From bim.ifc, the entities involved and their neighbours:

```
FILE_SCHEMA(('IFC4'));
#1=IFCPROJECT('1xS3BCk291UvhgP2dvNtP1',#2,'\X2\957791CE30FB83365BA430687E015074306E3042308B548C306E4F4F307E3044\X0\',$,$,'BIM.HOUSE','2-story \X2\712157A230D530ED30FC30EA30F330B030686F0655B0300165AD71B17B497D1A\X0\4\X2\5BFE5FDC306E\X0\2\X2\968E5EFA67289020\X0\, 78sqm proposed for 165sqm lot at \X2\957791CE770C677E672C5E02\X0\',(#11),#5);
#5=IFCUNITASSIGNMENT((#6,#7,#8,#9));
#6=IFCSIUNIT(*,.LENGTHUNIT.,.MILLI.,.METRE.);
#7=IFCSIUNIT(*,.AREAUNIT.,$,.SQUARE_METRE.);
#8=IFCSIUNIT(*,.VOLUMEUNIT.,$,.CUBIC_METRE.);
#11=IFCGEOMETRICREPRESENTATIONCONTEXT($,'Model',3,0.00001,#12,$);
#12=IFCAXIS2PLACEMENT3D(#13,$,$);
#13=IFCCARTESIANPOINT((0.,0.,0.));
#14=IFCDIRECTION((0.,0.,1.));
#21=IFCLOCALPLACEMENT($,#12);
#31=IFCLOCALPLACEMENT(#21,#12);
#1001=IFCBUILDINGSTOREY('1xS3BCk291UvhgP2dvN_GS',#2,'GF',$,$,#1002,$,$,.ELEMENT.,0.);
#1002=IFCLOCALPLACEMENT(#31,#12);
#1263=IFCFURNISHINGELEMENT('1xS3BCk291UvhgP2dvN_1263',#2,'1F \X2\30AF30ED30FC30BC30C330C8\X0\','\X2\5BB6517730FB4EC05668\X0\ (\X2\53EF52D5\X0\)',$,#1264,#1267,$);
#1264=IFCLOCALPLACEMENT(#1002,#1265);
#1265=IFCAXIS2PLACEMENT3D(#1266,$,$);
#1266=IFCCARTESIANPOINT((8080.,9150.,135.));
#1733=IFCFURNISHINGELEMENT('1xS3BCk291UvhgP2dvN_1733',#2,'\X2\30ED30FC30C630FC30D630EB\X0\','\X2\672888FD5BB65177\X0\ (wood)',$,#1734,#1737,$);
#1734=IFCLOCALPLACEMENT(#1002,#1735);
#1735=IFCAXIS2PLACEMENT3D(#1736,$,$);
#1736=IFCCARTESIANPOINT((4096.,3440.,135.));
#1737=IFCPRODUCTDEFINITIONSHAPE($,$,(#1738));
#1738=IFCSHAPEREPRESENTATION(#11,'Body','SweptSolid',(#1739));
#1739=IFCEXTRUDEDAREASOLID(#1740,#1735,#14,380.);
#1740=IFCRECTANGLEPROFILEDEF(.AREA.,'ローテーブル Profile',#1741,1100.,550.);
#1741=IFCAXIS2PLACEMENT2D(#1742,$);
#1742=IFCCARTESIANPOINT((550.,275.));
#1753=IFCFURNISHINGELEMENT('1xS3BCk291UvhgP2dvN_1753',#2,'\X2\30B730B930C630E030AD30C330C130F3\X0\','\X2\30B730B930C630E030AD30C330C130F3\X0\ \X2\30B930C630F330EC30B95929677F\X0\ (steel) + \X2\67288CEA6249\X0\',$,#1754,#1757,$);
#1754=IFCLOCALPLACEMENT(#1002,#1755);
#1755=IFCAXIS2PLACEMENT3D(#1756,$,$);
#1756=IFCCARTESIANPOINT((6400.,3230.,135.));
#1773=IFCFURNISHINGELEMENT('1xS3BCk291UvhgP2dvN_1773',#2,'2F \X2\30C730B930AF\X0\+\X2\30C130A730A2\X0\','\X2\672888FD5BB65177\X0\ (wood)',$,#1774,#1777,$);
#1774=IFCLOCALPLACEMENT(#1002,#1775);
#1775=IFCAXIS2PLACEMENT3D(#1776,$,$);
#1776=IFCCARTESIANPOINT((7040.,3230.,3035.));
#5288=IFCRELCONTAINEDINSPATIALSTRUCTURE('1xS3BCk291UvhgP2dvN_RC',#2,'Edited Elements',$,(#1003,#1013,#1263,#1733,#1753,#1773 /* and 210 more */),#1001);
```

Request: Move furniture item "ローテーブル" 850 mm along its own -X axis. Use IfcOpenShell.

```python
import ifcopenshell
import ifcopenshell.api.geometry
import ifcopenshell.util.placement

model = ifcopenshell.open("bim.ifc")

item = model.by_id(1733)
matrix = ifcopenshell.util.placement.get_local_placement(item.ObjectPlacement)
matrix[:3, 3] -= matrix[:3, 0] * 850.0
ifcopenshell.api.geometry.edit_object_placement(model, product=item, matrix=matrix, is_si=False)

print(ifcopenshell.util.placement.get_local_placement(item.ObjectPlacement).round(3) + 0.0)

model.write("bim-out.ifc")
```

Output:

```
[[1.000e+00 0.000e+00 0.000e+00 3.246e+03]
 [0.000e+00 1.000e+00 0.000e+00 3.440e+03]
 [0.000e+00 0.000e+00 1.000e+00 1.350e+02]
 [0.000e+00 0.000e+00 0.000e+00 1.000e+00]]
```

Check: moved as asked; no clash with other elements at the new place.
